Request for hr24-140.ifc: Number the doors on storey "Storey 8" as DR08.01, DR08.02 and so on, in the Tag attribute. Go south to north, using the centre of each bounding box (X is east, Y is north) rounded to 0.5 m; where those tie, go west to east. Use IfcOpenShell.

First a look at what the model holds.

```python
import ifcopenshell
import ifcopenshell.util.element
import ifcopenshell.util.placement

model = ifcopenshell.open("hr24-140.ifc")
print(model.schema)
storey = next(s for s in model.by_type("IfcBuildingStorey") if s.Name == "Storey 8")
doors = [e for e in ifcopenshell.util.element.get_decomposition(storey) if e.is_a("IfcDoor")]
for e in sorted(doors, key=lambda e: e.id()):
    origin = ifcopenshell.util.placement.get_local_placement(e.ObjectPlacement)[:3, 3]
    print(e.id(), e.Tag, e.Name, origin.round(2) + 0.0, sep=" | ")
```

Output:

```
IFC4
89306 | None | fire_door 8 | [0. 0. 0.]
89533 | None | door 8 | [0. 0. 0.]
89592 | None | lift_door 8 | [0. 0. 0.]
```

```python
import ifcopenshell
import ifcopenshell.geom
import ifcopenshell.util.element
import ifcopenshell.util.shape

model = ifcopenshell.open("hr24-140.ifc")
settings = ifcopenshell.geom.settings()
settings.set("use-world-coords", True)


def centre(element):
    shape = ifcopenshell.geom.create_shape(settings, element)
    return ifcopenshell.util.shape.get_bbox_centroid(shape.geometry)


storey = next(s for s in model.by_type("IfcBuildingStorey") if s.Name == "Storey 8")
doors = [e for e in ifcopenshell.util.element.get_decomposition(storey) if e.is_a("IfcDoor")]

# Insertion points can sit at a corner or the storey origin, so sort by the geometry (in metres).
centres = {e: centre(e) for e in doors}
doors.sort(key=lambda e: (round(centres[e][1] / 0.5), centres[e][0]))

for i, e in enumerate(doors, start=1):
    number = f"DR08.{i:02d}"
    e.Tag = number
    print(e.id(), number)

model.write("hr24-140_rev.ifc")
```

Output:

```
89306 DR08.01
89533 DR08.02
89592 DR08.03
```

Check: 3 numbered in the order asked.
